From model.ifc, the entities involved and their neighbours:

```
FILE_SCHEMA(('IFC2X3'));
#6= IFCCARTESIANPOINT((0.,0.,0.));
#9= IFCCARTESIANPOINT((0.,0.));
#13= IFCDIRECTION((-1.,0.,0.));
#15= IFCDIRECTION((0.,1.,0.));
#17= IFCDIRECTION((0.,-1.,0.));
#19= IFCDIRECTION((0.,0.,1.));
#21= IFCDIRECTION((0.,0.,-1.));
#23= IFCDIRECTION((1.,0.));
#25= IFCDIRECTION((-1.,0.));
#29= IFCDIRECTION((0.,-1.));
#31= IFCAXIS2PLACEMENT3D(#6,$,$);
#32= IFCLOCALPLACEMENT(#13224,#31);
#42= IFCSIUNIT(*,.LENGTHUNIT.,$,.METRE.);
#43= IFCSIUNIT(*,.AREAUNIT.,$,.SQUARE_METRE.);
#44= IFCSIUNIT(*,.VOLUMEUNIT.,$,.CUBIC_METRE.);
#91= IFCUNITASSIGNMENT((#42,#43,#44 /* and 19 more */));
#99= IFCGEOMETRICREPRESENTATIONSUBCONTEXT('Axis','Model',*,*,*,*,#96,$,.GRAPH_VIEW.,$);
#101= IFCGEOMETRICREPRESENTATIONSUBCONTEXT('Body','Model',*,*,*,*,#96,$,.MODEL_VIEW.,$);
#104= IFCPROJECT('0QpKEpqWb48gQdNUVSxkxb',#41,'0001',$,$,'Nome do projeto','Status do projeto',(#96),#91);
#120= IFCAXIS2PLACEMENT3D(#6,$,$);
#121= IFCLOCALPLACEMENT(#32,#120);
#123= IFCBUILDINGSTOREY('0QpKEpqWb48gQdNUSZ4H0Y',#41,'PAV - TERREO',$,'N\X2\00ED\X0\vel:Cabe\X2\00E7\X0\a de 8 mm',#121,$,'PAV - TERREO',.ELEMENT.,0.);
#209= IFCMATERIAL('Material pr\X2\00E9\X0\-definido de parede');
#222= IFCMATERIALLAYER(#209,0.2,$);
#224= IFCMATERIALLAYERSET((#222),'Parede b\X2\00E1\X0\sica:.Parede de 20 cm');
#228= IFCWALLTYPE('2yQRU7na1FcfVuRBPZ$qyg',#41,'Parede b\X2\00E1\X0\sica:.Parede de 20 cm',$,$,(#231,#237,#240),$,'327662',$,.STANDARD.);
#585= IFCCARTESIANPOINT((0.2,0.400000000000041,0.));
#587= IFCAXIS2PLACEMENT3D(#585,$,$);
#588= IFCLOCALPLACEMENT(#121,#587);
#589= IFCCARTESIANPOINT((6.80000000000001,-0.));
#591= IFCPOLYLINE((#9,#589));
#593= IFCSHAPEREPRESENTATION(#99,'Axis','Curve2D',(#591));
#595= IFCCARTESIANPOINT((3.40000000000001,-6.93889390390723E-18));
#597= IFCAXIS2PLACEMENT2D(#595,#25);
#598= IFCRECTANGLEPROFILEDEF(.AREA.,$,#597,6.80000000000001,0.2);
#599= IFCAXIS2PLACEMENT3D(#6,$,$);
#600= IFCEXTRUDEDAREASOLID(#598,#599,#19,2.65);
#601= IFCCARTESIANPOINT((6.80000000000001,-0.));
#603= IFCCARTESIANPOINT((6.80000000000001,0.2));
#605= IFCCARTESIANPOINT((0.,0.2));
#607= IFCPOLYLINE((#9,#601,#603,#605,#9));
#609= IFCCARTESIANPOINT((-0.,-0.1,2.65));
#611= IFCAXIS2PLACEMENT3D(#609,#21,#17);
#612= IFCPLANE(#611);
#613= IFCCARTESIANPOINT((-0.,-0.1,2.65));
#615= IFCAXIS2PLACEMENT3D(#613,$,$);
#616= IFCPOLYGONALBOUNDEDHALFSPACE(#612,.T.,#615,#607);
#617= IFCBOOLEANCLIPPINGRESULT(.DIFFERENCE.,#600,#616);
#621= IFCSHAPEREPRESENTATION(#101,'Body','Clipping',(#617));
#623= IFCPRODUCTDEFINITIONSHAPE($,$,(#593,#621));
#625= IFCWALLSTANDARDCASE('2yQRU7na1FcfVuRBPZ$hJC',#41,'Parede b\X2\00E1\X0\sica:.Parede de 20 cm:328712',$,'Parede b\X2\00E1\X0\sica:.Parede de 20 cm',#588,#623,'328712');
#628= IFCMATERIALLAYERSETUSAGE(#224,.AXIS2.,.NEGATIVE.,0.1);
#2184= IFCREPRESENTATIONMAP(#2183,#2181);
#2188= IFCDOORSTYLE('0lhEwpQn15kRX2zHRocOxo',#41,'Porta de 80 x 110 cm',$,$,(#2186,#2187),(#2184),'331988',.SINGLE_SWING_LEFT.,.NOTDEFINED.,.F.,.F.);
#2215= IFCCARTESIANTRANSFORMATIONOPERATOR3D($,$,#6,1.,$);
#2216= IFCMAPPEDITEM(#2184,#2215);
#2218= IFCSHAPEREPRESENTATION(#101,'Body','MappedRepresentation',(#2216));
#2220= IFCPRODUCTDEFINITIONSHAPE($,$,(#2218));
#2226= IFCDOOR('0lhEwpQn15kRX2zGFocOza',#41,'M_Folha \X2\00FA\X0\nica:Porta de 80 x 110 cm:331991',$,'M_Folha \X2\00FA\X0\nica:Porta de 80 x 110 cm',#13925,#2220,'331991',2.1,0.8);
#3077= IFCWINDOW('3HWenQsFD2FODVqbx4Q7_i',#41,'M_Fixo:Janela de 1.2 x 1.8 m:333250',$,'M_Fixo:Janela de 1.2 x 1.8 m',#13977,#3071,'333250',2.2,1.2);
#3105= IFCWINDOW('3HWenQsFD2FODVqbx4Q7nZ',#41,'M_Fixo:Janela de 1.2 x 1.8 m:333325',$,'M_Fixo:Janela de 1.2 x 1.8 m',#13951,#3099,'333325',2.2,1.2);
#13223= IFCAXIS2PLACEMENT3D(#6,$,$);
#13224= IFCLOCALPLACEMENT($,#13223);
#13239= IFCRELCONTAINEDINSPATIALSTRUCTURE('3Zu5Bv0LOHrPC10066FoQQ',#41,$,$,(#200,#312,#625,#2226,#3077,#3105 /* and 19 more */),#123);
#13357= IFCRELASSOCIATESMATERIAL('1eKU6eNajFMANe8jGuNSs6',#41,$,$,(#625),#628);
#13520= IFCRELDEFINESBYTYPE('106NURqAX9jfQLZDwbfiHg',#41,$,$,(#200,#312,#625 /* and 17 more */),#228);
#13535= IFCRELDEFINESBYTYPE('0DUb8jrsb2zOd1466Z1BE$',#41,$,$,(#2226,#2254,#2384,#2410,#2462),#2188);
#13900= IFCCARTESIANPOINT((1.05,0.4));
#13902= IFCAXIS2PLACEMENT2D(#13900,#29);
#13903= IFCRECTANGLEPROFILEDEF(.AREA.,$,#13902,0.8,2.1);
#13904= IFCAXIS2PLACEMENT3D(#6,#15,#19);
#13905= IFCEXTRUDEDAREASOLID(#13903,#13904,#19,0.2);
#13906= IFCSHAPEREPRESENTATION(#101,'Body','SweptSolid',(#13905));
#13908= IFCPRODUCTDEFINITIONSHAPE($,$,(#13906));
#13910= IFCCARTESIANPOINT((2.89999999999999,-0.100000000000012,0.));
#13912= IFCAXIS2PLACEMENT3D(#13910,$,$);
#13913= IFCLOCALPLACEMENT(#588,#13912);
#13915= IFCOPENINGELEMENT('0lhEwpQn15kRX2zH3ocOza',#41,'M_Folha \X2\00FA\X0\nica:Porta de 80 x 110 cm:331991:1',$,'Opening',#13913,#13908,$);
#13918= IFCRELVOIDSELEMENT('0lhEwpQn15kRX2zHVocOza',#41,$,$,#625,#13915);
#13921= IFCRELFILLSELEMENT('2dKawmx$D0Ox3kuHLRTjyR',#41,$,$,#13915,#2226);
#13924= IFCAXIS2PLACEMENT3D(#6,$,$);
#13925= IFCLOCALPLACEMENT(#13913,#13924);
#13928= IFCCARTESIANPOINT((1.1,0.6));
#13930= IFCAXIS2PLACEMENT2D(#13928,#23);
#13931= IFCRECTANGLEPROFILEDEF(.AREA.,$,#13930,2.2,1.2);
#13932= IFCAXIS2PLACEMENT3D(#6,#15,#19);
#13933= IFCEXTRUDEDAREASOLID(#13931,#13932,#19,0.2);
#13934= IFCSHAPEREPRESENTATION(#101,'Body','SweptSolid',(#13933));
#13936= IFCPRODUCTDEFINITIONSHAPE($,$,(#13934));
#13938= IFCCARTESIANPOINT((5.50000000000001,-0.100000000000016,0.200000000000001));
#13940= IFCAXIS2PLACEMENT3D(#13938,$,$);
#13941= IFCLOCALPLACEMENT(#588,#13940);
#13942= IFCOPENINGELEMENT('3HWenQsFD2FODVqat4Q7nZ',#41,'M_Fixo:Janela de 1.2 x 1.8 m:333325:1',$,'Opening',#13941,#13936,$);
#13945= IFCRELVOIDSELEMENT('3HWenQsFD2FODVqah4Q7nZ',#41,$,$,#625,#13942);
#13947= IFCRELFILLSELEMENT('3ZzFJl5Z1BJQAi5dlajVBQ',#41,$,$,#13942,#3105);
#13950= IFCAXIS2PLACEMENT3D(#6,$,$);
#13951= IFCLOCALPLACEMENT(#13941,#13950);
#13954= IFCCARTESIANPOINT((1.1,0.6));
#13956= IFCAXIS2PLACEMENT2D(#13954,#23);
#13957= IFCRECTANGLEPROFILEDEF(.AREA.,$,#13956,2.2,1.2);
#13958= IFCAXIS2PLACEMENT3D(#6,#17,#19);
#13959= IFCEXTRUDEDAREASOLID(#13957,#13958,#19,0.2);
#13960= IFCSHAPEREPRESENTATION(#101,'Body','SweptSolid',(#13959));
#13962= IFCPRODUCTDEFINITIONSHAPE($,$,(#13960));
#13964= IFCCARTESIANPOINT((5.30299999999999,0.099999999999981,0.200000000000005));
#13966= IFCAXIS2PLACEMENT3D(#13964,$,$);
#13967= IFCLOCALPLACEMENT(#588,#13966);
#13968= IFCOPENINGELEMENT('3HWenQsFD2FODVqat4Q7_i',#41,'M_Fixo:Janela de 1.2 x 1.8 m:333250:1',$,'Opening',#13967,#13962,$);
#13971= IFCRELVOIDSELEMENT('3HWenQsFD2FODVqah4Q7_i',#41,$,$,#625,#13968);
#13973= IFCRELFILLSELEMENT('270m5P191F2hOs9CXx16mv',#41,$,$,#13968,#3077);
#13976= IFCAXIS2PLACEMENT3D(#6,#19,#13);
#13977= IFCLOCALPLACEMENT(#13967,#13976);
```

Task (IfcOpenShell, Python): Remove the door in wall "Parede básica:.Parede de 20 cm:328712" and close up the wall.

```python
import ifcopenshell
import ifcopenshell.api.feature
import ifcopenshell.api.root
import ifcopenshell.geom
import ifcopenshell.util.shape

model = ifcopenshell.open("model.ifc")
settings = ifcopenshell.geom.settings()


def volume(element):
    """Net volume in cubic metres, openings subtracted."""
    shape = ifcopenshell.geom.create_shape(settings, element)
    return ifcopenshell.util.shape.get_volume(shape.geometry)


door = model.by_guid("0lhEwpQn15kRX2zGFocOza")
opening = door.FillsVoids[0].RelatingOpeningElement
wall = opening.VoidsElements[0].RelatingBuildingElement
before = volume(wall)

ifcopenshell.api.root.remove_product(model, product=door)
ifcopenshell.api.feature.remove_feature(model, feature=opening)

after = volume(wall)

print(f"wall volume {before:.3f} -> {after:.3f} m3")

model.write("model_rev.ifc")
```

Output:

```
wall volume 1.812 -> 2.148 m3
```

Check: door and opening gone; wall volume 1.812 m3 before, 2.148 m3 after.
